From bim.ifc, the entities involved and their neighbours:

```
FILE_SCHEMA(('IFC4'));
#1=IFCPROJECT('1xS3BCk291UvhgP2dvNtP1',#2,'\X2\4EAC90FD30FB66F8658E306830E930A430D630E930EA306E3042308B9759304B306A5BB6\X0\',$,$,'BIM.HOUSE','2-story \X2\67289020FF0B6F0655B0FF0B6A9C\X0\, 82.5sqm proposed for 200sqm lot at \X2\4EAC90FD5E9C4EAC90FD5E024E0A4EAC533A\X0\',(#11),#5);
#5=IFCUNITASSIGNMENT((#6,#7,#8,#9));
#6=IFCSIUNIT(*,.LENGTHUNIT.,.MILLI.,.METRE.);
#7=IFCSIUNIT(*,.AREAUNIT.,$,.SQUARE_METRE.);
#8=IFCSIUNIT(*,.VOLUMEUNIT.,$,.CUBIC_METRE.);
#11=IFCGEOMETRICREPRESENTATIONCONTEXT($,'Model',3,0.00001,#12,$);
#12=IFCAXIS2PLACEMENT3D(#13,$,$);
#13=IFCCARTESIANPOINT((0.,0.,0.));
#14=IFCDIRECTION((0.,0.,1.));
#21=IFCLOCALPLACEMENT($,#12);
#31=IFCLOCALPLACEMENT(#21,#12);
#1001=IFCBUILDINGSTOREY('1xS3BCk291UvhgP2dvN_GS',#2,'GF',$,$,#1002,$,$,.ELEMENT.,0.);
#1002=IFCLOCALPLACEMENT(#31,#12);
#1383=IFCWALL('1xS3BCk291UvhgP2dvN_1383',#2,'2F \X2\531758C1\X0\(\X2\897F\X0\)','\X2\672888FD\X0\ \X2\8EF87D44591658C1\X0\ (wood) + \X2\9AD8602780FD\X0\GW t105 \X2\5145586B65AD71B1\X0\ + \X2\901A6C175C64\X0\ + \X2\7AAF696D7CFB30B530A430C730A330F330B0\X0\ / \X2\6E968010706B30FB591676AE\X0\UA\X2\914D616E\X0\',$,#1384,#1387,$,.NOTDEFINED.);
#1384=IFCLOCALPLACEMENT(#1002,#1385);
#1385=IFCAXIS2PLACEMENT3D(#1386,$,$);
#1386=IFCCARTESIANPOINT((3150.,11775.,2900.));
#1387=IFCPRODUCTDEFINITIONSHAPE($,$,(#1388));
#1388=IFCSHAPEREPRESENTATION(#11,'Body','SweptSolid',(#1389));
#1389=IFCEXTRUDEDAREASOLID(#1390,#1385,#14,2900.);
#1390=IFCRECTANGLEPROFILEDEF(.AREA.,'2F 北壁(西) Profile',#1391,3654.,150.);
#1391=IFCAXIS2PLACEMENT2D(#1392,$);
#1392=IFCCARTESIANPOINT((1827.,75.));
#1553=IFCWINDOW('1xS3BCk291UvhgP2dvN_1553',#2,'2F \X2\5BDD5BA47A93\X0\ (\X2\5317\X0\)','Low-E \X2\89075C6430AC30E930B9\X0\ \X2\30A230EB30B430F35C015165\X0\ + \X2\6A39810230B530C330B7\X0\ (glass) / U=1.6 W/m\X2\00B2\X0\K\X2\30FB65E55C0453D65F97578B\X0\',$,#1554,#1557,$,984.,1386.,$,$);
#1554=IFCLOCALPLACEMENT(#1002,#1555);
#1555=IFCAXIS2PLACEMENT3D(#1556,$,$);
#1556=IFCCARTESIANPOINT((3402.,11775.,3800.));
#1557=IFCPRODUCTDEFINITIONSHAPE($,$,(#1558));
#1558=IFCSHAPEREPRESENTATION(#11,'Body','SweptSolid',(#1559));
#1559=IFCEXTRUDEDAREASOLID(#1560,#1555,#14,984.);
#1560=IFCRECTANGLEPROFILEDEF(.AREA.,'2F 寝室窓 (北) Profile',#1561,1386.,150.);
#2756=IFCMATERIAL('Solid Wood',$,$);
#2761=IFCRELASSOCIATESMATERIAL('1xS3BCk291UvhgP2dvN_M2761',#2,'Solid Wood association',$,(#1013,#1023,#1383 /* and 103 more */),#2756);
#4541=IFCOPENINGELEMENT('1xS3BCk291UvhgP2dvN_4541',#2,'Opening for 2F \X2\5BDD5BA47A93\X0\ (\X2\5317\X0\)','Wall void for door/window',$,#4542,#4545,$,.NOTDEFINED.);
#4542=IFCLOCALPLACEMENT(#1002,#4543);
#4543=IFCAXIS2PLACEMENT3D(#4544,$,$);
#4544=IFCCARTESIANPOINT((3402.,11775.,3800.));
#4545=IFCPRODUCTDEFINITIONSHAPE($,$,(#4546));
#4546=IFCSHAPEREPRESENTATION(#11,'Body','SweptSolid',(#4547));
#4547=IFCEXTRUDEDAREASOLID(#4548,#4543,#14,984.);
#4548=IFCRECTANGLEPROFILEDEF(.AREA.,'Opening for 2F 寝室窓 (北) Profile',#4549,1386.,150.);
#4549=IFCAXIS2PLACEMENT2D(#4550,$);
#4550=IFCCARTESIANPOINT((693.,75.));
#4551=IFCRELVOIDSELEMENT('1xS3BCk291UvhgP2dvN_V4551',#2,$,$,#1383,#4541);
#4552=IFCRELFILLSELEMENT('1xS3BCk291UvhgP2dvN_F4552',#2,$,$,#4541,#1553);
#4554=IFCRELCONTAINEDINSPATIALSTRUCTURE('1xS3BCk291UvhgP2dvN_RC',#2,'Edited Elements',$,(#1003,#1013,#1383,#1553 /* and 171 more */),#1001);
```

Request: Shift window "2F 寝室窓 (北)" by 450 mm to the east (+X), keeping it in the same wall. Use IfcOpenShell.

```python
import ifcopenshell
import ifcopenshell.api.geometry
import ifcopenshell.util.placement
import ifcopenshell.util.unit

model = ifcopenshell.open("bim.ifc")
unit_scale = ifcopenshell.util.unit.calculate_unit_scale(model)

window = model.by_guid("1xS3BCk291UvhgP2dvN_1553")
opening = window.FillsVoids[0].RelatingOpeningElement
wall = opening.VoidsElements[0].RelatingBuildingElement

wall_matrix = ifcopenshell.util.placement.get_local_placement(wall.ObjectPlacement)
shift = wall_matrix[:3, 0] * 0.45 / unit_scale
before = ifcopenshell.util.placement.get_local_placement(window.ObjectPlacement)[:3, 3].copy()

# The window is not placed relative to its opening, so move both.
for product in (opening, window):
    matrix = ifcopenshell.util.placement.get_local_placement(product.ObjectPlacement)
    matrix[:3, 3] += shift
    ifcopenshell.api.geometry.edit_object_placement(model, product=product, matrix=matrix, is_si=False)

after = ifcopenshell.util.placement.get_local_placement(window.ObjectPlacement)[:3, 3]
print("window moved by", (after - before).round(3) + 0.0)

model.write("bim_rev.ifc")
```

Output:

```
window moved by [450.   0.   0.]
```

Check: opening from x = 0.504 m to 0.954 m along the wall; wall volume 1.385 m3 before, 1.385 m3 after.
